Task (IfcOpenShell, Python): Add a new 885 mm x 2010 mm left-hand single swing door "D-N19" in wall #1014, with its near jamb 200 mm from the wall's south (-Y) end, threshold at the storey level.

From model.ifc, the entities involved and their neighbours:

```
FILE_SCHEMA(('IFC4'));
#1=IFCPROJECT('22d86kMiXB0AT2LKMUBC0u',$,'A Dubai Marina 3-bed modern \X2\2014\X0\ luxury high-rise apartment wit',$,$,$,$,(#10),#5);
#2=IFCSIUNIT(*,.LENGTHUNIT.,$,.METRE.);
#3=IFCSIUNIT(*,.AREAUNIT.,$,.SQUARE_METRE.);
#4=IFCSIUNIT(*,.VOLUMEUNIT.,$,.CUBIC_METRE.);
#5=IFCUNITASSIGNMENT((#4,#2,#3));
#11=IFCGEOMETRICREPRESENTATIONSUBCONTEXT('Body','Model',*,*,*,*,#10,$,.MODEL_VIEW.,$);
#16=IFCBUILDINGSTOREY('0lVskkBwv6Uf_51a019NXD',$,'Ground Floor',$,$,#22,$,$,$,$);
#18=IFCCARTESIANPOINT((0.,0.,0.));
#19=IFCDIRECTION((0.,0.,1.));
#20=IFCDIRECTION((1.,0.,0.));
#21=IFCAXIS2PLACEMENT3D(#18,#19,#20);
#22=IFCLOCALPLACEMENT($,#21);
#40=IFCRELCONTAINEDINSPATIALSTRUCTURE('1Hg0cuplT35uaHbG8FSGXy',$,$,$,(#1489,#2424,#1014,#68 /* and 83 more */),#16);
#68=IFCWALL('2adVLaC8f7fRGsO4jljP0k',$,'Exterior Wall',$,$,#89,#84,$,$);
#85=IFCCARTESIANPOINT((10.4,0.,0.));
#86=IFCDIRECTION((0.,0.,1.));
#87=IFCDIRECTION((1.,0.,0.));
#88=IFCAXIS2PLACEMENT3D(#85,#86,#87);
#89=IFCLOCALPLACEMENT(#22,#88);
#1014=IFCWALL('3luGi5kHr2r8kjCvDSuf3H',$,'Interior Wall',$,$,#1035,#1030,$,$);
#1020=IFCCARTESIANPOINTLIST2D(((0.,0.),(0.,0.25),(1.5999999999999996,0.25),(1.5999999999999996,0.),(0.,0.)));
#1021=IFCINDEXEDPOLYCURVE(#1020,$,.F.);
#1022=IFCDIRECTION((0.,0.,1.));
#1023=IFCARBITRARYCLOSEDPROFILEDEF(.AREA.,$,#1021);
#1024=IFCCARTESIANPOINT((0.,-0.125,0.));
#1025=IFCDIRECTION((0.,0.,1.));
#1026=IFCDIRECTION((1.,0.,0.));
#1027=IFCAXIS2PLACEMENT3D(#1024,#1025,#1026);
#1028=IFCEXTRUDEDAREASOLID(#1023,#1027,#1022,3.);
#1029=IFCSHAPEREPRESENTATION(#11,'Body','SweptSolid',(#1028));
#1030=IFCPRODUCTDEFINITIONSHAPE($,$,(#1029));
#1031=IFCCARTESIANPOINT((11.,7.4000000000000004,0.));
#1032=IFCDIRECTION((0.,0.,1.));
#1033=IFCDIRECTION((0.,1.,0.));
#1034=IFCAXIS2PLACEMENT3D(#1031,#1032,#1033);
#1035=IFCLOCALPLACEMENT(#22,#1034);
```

```python
import numpy as np
import ifcopenshell
import ifcopenshell.api.feature
import ifcopenshell.api.geometry
import ifcopenshell.api.root
import ifcopenshell.api.spatial
import ifcopenshell.geom
import ifcopenshell.util.element
import ifcopenshell.util.placement
import ifcopenshell.util.representation
import ifcopenshell.util.shape
import ifcopenshell.util.unit

model = ifcopenshell.open("model.ifc")
unit_scale = ifcopenshell.util.unit.calculate_unit_scale(model)
settings = ifcopenshell.geom.settings()


def volume(element):
    """Net volume in cubic metres, openings subtracted."""
    shape = ifcopenshell.geom.create_shape(settings, element)
    return ifcopenshell.util.shape.get_volume(shape.geometry)


wall = model.by_guid("3luGi5kHr2r8kjCvDSuf3H")
storey = ifcopenshell.util.element.get_container(wall, ifc_class="IfcBuildingStorey")
context = ifcopenshell.util.representation.get_context(model, "Model", "Body", "MODEL_VIEW")
before = volume(wall)

width, height, from_end, sill = 0.885, 2.01, 0.2, 0.0  # metres

# The wall runs along its own X axis, and the end named is its -X end.
wall_shape = ifcopenshell.geom.create_shape(settings, wall)
x, y, z = ifcopenshell.util.shape.get_vertices(wall_shape.geometry).T
start = x.min() + from_end
face, thickness = float(y.min()), float(y.max() - y.min())
wall_matrix = ifcopenshell.util.placement.get_local_placement(wall.ObjectPlacement)
level = ifcopenshell.util.placement.get_local_placement(storey.ObjectPlacement)[2, 3]


def in_wall(x, y):
    """Placement at x, y metres in the wall's axes, at sill height."""
    matrix = wall_matrix.copy()
    matrix[:, 3] = wall_matrix @ np.array([x / unit_scale, y / unit_scale, 0.0, 1.0])
    matrix[2, 3] = level + sill / unit_scale
    return matrix


# Opening: a box that overshoots both wall faces by 50 mm.
opening = ifcopenshell.api.root.create_entity(model, ifc_class="IfcOpeningElement", predefined_type="OPENING")
box = ifcopenshell.api.geometry.add_wall_representation(
    model, context=context, length=width, height=height, thickness=thickness + 0.1
)
ifcopenshell.api.geometry.assign_representation(model, product=opening, representation=box)
ifcopenshell.api.geometry.edit_object_placement(model, product=opening, matrix=in_wall(start, face - 0.05), is_si=False)
ifcopenshell.api.feature.add_feature(model, feature=opening, element=wall)

door = ifcopenshell.api.root.create_entity(model, ifc_class="IfcDoor", name="D-N19", predefined_type="DOOR")
door.OverallWidth, door.OverallHeight = width / unit_scale, height / unit_scale
door.OperationType = "SINGLE_SWING_LEFT"
body = ifcopenshell.api.geometry.add_door_representation(
    model,
    context=context,
    overall_width=door.OverallWidth,
    overall_height=door.OverallHeight,
    operation_type="SINGLE_SWING_LEFT",
    lining_properties={"LiningDepth": thickness / unit_scale, "ThresholdDepth": thickness / unit_scale},
)
ifcopenshell.api.geometry.assign_representation(model, product=door, representation=body)
ifcopenshell.api.spatial.assign_container(model, products=[door], relating_structure=storey)
ifcopenshell.api.feature.add_filling(model, opening=opening, element=door)

# The lining spans the wall, so the door starts at the wall face.
ifcopenshell.api.geometry.edit_object_placement(model, product=door, matrix=in_wall(start, face), is_si=False)

after = volume(wall)

print(f"wall volume {before:.3f} -> {after:.3f} m3")

model.write("model-out.ifc")
```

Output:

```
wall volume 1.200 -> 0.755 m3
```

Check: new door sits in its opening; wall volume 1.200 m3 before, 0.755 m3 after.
